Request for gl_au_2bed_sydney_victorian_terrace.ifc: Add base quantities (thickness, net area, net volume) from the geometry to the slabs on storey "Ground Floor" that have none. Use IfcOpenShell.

First a look at what the model holds.

```python
import ifcopenshell
import ifcopenshell.util.element
import ifcopenshell.util.unit

model = ifcopenshell.open("gl_au_2bed_sydney_victorian_terrace.ifc")
print(model.schema)
for unit_type in ("LENGTHUNIT", "AREAUNIT", "VOLUMEUNIT"):
    print(unit_type, ifcopenshell.util.unit.calculate_unit_scale(model, unit_type))
storey = next(s for s in model.by_type("IfcBuildingStorey") if s.Name == "Ground Floor")
slabs = [e for e in ifcopenshell.util.element.get_decomposition(storey) if e.is_a("IfcSlab")]
for e in sorted(slabs, key=lambda e: e.id()):
    print(e.id(), e.is_a(), e.Name, list(ifcopenshell.util.element.get_psets(e, qtos_only=True)), sep=" | ")
```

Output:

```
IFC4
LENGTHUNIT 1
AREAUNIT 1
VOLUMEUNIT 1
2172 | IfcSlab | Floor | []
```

```python
import ifcopenshell
import ifcopenshell.api.pset
import ifcopenshell.geom
import ifcopenshell.util.element
import ifcopenshell.util.shape
import ifcopenshell.util.unit

model = ifcopenshell.open("gl_au_2bed_sydney_victorian_terrace.ifc")
unit_scale = ifcopenshell.util.unit.calculate_unit_scale(model)
area_scale = ifcopenshell.util.unit.calculate_unit_scale(model, "AREAUNIT")
volume_scale = ifcopenshell.util.unit.calculate_unit_scale(model, "VOLUMEUNIT")
settings = ifcopenshell.geom.settings()

storey = next(s for s in model.by_type("IfcBuildingStorey") if s.Name == "Ground Floor")
slabs = [e for e in ifcopenshell.util.element.get_decomposition(storey) if e.is_a("IfcSlab")]

for e in sorted(slabs, key=lambda e: e.id()):
    if ifcopenshell.util.element.get_psets(e, qtos_only=True, should_inherit=False):
        continue
    # Geometry comes back in metres, in the element's own axes.
    shape = ifcopenshell.geom.create_shape(settings, e)
    values = {
        "Width": ifcopenshell.util.shape.get_z(shape.geometry) / unit_scale,
        "NetArea": ifcopenshell.util.shape.get_footprint_area(shape.geometry) / area_scale,
        "NetVolume": ifcopenshell.util.shape.get_volume(shape.geometry) / volume_scale,
    }
    qto = ifcopenshell.api.pset.add_qto(model, product=e, name="Qto_SlabBaseQuantities")
    ifcopenshell.api.pset.edit_qto(model, qto=qto, properties=values)
    print(e.id(), {k: round(v, 3) for k, v in values.items()})

model.write("gl_au_2bed_sydney_victorian_terrace_rev.ifc")
```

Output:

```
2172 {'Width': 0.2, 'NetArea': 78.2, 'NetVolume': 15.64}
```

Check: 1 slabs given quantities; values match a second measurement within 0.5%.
